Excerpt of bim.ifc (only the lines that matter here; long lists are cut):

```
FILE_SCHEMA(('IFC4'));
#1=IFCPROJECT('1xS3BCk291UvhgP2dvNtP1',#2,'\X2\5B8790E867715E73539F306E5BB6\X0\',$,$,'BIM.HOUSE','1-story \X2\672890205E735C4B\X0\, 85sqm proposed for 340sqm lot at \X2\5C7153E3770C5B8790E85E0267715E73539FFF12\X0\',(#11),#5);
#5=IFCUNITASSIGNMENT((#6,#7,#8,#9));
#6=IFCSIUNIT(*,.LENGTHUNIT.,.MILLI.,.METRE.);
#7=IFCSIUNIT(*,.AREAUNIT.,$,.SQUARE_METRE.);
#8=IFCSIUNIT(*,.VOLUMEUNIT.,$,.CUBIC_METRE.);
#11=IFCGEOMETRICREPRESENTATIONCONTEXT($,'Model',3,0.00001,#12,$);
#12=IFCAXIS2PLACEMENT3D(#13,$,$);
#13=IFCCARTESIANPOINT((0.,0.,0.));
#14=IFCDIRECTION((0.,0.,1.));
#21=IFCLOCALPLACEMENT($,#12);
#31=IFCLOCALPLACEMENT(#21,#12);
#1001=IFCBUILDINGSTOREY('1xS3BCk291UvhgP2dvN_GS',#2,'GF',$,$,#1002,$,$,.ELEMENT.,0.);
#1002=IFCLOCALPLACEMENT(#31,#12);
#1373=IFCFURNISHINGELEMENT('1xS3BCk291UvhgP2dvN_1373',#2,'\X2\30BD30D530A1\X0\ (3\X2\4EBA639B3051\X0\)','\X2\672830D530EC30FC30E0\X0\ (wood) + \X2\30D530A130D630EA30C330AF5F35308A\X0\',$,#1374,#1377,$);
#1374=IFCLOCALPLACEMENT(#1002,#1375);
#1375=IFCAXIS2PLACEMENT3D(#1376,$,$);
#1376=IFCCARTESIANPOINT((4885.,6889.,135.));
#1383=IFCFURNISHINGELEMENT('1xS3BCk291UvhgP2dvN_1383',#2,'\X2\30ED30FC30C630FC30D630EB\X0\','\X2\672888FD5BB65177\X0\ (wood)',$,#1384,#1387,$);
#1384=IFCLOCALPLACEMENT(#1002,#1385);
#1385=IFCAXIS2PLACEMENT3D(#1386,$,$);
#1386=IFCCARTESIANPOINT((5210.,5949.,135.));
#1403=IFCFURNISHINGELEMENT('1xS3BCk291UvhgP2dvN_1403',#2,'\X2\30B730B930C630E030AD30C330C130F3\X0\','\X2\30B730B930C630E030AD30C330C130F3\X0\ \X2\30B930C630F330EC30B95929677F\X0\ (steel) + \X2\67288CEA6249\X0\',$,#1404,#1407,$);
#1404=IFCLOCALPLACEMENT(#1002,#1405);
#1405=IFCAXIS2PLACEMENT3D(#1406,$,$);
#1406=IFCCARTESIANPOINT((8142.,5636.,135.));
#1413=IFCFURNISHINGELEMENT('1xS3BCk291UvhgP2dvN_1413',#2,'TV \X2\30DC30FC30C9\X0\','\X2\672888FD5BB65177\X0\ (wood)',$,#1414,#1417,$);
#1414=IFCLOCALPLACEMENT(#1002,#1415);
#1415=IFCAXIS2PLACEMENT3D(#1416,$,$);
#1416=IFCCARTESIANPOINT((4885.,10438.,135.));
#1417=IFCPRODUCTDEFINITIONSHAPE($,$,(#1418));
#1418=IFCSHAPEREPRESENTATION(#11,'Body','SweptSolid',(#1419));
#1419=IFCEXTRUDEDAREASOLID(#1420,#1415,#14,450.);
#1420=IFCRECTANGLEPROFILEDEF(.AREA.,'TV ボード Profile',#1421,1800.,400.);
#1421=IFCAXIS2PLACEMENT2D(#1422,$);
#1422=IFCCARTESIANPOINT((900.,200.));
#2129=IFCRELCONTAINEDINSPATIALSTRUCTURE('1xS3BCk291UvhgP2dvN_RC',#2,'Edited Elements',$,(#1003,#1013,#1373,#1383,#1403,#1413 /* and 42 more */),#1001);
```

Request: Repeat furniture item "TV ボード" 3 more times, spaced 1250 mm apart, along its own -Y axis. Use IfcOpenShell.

```python
import ifcopenshell
import ifcopenshell.api.geometry
import ifcopenshell.api.root
import ifcopenshell.util.element
import ifcopenshell.util.placement
import ifcopenshell.util.unit

model = ifcopenshell.open("bim.ifc")
unit_scale = ifcopenshell.util.unit.calculate_unit_scale(model)


def reuse_history(source, copy):
    """copy_class also copies each property set's owner history, people and application; keep the originals."""
    for rel in copy.IsDefinedBy:
        if rel.is_a("IfcRelDefinesByProperties") and (history := rel.RelatingPropertyDefinition.OwnerHistory):
            rel.RelatingPropertyDefinition.OwnerHistory = source.OwnerHistory
            ifcopenshell.util.element.remove_deep2(model, history)


source = model.by_guid("1xS3BCk291UvhgP2dvN_1413")
base = ifcopenshell.util.placement.get_local_placement(source.ObjectPlacement)
step = -base[:3, 1] * 1.25 / unit_scale

for i in range(1, 4):
    copy = ifcopenshell.api.root.copy_class(model, product=source)
    copy.Representation = ifcopenshell.util.element.copy_deep(
        model, source.Representation, exclude=["IfcGeometricRepresentationContext", "IfcRepresentationMap"]
    )
    reuse_history(source, copy)
    matrix = base.copy()
    matrix[:3, 3] += i * step
    print("added at", matrix[:3, 3].round(3) + 0.0)
    ifcopenshell.api.geometry.edit_object_placement(model, product=copy, matrix=matrix, is_si=False)

model.write("bim-out.ifc")
```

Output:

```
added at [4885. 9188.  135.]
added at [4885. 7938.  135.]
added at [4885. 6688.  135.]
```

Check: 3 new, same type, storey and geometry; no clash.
